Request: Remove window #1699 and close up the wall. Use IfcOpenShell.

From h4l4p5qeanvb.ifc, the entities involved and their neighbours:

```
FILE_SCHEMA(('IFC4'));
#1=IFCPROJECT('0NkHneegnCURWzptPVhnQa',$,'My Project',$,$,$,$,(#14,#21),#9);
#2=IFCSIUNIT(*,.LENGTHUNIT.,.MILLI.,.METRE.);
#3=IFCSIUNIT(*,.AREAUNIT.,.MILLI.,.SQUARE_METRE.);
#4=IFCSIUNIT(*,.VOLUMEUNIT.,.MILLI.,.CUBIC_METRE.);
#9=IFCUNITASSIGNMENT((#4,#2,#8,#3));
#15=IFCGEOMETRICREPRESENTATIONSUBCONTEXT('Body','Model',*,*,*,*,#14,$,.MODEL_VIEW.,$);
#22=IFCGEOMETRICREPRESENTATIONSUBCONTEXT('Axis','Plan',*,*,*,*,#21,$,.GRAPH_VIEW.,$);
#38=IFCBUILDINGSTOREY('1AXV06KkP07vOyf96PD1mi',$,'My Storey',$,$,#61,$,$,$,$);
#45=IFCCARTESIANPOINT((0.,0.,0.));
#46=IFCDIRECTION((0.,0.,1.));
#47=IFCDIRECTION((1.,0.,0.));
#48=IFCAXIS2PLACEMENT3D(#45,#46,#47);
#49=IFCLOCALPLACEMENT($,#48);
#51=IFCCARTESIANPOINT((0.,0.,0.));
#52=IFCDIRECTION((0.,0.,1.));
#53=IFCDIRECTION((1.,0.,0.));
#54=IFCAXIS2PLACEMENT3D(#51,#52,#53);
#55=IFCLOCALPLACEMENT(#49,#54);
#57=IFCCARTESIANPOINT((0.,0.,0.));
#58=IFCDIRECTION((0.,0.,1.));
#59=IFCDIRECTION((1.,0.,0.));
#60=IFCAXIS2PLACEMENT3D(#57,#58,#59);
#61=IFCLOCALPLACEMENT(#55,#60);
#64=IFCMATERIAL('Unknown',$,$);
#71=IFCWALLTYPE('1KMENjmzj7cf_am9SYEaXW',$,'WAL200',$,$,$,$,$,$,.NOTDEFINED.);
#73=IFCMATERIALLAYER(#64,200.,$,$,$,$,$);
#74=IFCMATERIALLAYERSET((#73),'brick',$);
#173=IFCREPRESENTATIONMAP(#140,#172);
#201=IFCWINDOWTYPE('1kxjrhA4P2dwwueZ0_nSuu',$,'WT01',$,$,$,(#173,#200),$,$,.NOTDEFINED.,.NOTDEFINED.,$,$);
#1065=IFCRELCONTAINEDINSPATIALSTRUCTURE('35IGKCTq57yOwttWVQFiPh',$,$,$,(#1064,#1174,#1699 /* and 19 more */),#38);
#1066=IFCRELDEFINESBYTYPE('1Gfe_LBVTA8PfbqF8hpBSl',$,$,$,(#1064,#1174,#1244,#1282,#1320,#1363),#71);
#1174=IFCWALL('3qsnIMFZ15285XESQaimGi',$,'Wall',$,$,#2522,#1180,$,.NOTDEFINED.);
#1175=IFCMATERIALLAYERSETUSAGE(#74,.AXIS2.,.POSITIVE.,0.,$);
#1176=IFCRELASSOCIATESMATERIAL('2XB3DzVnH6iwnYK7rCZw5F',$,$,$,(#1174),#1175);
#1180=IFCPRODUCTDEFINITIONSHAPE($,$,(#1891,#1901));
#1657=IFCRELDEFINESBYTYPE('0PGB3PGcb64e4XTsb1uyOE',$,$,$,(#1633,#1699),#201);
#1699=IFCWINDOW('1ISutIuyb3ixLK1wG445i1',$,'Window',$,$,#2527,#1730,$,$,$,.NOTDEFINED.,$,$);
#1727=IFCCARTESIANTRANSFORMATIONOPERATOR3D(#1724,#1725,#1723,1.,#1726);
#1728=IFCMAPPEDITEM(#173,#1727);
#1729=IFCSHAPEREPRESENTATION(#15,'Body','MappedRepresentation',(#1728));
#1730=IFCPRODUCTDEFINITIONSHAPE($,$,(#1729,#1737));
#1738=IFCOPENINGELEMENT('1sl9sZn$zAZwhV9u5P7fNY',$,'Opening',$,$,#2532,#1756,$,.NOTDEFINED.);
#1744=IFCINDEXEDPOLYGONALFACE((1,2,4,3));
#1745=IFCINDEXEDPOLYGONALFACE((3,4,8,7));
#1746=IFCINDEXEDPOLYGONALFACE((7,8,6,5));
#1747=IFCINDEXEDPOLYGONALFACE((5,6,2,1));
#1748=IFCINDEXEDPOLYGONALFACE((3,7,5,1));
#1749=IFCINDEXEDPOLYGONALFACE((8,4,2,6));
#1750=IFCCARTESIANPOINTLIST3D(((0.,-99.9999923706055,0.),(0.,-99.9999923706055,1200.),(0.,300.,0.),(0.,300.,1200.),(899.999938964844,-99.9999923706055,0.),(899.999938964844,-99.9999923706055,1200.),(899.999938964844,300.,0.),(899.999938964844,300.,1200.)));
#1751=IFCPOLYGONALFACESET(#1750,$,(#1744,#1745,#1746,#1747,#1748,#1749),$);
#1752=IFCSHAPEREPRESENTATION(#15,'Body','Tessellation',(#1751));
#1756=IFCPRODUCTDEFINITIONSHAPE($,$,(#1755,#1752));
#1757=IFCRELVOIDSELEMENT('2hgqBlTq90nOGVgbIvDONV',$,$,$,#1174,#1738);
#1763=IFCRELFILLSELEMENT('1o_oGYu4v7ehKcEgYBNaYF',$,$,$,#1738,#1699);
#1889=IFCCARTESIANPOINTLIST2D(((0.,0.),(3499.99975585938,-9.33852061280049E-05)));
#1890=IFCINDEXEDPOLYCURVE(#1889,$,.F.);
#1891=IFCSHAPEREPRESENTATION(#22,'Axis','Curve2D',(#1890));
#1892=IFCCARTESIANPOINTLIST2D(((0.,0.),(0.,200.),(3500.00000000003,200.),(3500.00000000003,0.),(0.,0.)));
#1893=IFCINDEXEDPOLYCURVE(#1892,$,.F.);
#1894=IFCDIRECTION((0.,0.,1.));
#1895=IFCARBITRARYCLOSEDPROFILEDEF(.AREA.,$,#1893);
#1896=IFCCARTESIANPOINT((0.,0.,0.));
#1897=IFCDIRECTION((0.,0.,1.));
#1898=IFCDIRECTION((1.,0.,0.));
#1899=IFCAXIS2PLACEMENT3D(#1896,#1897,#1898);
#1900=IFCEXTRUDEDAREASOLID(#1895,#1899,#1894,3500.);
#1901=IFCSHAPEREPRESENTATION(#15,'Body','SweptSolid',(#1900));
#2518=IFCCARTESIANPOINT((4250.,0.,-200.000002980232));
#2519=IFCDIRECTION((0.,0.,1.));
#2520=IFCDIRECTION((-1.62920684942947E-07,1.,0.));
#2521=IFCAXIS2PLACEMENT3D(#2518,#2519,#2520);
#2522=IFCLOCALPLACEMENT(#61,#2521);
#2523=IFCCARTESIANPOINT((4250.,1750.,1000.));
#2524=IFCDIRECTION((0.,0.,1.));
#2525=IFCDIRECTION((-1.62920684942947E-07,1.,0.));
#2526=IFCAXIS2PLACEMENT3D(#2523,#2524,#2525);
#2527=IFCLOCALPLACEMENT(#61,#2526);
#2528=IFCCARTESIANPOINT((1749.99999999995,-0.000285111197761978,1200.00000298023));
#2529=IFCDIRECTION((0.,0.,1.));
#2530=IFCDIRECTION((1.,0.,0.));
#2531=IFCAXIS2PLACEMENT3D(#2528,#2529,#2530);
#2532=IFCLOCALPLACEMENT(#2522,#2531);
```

```python
import ifcopenshell
import ifcopenshell.api.feature
import ifcopenshell.api.root
import ifcopenshell.geom
import ifcopenshell.util.shape

model = ifcopenshell.open("h4l4p5qeanvb.ifc")
settings = ifcopenshell.geom.settings()


def volume(element):
    """Net volume in cubic metres, openings subtracted."""
    shape = ifcopenshell.geom.create_shape(settings, element)
    return ifcopenshell.util.shape.get_volume(shape.geometry)


window = model.by_id(1699)
opening = window.FillsVoids[0].RelatingOpeningElement
wall = opening.VoidsElements[0].RelatingBuildingElement
before = volume(wall)

ifcopenshell.api.root.remove_product(model, product=window)
ifcopenshell.api.feature.remove_feature(model, feature=opening)

after = volume(wall)

print(f"wall volume {before:.3f} -> {after:.3f} m3")

model.write("h4l4p5qeanvb_updated.ifc")
```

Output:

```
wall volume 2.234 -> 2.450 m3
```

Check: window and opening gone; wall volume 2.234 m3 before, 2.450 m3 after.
